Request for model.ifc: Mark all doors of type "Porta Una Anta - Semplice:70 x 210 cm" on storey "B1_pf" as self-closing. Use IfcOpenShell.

First a look at what the model holds.

```python
import ifcopenshell
import ifcopenshell.util.element

model = ifcopenshell.open("model.ifc")
print(model.schema)
storey = next(s for s in model.by_type("IfcBuildingStorey") if s.Name == "B1_pf")
doors = [e for e in ifcopenshell.util.element.get_decomposition(storey) if e.is_a("IfcDoor")]
seen = {}
for e in doors:
    element_type = ifcopenshell.util.element.get_type(e)
    key = (element_type.Name if element_type != e and element_type else None, ifcopenshell.util.element.get_pset(e, "Pset_DoorCommon", "SelfClosing"))
    seen[key] = seen.get(key, 0) + 1
for (name, value), count in sorted(seen.items(), key=str):
    print(count, "x", name, "|", value)
```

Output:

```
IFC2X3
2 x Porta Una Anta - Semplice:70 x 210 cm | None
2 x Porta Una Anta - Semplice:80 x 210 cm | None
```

```python
import ifcopenshell
import ifcopenshell.api.pset
import ifcopenshell.util.element

model = ifcopenshell.open("model.ifc")

storey = next(s for s in model.by_type("IfcBuildingStorey") if s.Name == "B1_pf")
doors = [e for e in ifcopenshell.util.element.get_decomposition(storey) if e.is_a("IfcDoor")]

count = 0
for e in doors:
    element_type = ifcopenshell.util.element.get_type(e)
    if element_type in (None, e) or element_type.Name != "Porta Una Anta - Semplice:70 x 210 cm":
        continue
    # add_pset returns the element's existing set when there is one.
    pset = ifcopenshell.api.pset.add_pset(model, product=e, name="Pset_DoorCommon")
    ifcopenshell.api.pset.edit_pset(model, pset=pset, properties={"SelfClosing": True})
    count += 1

print(count, "doors updated")

model.write("model_rev.ifc")
```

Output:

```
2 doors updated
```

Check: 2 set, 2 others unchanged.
